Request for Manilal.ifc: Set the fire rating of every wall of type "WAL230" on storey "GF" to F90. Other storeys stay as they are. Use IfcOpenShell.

First a look at what the model holds.

```python
import ifcopenshell
import ifcopenshell.util.element

model = ifcopenshell.open("Manilal.ifc")
print(model.schema)
storey = next(s for s in model.by_type("IfcBuildingStorey") if s.Name == "GF")
walls = [e for e in ifcopenshell.util.element.get_decomposition(storey) if e.is_a("IfcWall")]
seen = {}
for e in walls:
    element_type = ifcopenshell.util.element.get_type(e)
    key = (element_type.Name if element_type != e and element_type else None, ifcopenshell.util.element.get_pset(e, "Pset_WallCommon", "FireRating"))
    seen[key] = seen.get(key, 0) + 1
for (name, value), count in sorted(seen.items(), key=str):
    print(count, "x", name, "|", value)
```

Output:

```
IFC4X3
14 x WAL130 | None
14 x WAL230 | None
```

```python
import ifcopenshell
import ifcopenshell.api.pset
import ifcopenshell.util.element

model = ifcopenshell.open("Manilal.ifc")

storey = next(s for s in model.by_type("IfcBuildingStorey") if s.Name == "GF")
walls = [e for e in ifcopenshell.util.element.get_decomposition(storey) if e.is_a("IfcWall")]

count = 0
for e in walls:
    element_type = ifcopenshell.util.element.get_type(e)
    if element_type in (None, e) or element_type.Name != "WAL230":
        continue
    # add_pset returns the element's existing set when there is one.
    pset = ifcopenshell.api.pset.add_pset(model, product=e, name="Pset_WallCommon")
    ifcopenshell.api.pset.edit_pset(model, pset=pset, properties={"FireRating": "F90"})
    count += 1

print(count, "walls updated")

model.write("Manilal-out.ifc")
```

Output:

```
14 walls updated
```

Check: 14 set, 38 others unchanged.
